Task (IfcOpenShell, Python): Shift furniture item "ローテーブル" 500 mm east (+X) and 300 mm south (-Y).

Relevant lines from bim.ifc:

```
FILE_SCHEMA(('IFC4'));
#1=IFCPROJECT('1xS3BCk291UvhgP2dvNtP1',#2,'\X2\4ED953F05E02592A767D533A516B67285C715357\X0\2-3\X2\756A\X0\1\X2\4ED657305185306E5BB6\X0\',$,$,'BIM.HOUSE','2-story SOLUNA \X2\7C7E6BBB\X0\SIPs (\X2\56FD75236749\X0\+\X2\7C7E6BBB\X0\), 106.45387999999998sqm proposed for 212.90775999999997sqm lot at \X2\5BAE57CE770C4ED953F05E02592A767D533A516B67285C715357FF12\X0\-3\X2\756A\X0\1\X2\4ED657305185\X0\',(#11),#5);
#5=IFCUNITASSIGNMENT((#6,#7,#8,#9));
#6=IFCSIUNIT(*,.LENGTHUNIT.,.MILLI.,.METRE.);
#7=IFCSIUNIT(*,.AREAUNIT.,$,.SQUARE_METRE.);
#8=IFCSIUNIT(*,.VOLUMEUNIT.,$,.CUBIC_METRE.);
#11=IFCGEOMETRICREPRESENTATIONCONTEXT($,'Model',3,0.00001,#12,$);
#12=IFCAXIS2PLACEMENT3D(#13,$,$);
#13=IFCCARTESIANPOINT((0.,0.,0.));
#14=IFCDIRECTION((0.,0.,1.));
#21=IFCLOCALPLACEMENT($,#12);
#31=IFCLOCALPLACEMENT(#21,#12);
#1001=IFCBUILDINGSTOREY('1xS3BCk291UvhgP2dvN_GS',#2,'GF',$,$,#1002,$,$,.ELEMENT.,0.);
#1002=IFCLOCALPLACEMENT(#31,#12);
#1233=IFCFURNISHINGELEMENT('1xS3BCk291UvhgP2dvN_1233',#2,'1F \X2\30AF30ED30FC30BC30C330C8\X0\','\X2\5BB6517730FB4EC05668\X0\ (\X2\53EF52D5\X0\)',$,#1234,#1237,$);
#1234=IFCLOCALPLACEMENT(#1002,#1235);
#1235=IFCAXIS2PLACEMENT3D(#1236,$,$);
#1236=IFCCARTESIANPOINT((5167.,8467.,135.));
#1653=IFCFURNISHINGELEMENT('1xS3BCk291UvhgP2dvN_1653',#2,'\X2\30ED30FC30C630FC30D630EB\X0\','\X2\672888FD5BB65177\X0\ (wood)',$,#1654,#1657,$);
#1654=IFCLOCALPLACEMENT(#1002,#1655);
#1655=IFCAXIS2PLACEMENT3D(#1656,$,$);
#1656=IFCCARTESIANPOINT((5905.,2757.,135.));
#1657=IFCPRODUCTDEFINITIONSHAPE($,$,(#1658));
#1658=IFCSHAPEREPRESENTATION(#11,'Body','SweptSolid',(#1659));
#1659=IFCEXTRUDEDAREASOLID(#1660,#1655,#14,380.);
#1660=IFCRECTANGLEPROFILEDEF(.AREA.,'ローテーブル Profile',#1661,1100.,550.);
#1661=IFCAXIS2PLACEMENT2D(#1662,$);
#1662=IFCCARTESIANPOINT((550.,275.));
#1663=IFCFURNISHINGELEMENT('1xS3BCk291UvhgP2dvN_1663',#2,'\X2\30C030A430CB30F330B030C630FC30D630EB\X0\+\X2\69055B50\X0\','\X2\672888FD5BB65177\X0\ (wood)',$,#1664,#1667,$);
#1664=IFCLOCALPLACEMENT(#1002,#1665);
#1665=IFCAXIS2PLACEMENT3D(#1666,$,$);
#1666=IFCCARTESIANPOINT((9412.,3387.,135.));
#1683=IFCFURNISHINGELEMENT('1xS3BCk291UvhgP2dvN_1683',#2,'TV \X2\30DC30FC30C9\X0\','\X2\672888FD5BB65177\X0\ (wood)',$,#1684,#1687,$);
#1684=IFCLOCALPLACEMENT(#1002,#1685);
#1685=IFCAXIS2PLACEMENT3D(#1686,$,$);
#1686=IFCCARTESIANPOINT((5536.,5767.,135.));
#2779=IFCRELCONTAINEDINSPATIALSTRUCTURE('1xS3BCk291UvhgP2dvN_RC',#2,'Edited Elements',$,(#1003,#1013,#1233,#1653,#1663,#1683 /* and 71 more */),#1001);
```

```python
import ifcopenshell
import ifcopenshell.api.geometry
import ifcopenshell.util.placement
import ifcopenshell.util.unit

model = ifcopenshell.open("bim.ifc")
unit_scale = ifcopenshell.util.unit.calculate_unit_scale(model)

item = model.by_guid("1xS3BCk291UvhgP2dvN_1653")
matrix = ifcopenshell.util.placement.get_local_placement(item.ObjectPlacement)
matrix[0, 3] += 0.5 / unit_scale
matrix[1, 3] -= 0.3 / unit_scale
ifcopenshell.api.geometry.edit_object_placement(model, product=item, matrix=matrix, is_si=False)

print(ifcopenshell.util.placement.get_local_placement(item.ObjectPlacement).round(3) + 0.0)

model.write("bim_rev.ifc")
```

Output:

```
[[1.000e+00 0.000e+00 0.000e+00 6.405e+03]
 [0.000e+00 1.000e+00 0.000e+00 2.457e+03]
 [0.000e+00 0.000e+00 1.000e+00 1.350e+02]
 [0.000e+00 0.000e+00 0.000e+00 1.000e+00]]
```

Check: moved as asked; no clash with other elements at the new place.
